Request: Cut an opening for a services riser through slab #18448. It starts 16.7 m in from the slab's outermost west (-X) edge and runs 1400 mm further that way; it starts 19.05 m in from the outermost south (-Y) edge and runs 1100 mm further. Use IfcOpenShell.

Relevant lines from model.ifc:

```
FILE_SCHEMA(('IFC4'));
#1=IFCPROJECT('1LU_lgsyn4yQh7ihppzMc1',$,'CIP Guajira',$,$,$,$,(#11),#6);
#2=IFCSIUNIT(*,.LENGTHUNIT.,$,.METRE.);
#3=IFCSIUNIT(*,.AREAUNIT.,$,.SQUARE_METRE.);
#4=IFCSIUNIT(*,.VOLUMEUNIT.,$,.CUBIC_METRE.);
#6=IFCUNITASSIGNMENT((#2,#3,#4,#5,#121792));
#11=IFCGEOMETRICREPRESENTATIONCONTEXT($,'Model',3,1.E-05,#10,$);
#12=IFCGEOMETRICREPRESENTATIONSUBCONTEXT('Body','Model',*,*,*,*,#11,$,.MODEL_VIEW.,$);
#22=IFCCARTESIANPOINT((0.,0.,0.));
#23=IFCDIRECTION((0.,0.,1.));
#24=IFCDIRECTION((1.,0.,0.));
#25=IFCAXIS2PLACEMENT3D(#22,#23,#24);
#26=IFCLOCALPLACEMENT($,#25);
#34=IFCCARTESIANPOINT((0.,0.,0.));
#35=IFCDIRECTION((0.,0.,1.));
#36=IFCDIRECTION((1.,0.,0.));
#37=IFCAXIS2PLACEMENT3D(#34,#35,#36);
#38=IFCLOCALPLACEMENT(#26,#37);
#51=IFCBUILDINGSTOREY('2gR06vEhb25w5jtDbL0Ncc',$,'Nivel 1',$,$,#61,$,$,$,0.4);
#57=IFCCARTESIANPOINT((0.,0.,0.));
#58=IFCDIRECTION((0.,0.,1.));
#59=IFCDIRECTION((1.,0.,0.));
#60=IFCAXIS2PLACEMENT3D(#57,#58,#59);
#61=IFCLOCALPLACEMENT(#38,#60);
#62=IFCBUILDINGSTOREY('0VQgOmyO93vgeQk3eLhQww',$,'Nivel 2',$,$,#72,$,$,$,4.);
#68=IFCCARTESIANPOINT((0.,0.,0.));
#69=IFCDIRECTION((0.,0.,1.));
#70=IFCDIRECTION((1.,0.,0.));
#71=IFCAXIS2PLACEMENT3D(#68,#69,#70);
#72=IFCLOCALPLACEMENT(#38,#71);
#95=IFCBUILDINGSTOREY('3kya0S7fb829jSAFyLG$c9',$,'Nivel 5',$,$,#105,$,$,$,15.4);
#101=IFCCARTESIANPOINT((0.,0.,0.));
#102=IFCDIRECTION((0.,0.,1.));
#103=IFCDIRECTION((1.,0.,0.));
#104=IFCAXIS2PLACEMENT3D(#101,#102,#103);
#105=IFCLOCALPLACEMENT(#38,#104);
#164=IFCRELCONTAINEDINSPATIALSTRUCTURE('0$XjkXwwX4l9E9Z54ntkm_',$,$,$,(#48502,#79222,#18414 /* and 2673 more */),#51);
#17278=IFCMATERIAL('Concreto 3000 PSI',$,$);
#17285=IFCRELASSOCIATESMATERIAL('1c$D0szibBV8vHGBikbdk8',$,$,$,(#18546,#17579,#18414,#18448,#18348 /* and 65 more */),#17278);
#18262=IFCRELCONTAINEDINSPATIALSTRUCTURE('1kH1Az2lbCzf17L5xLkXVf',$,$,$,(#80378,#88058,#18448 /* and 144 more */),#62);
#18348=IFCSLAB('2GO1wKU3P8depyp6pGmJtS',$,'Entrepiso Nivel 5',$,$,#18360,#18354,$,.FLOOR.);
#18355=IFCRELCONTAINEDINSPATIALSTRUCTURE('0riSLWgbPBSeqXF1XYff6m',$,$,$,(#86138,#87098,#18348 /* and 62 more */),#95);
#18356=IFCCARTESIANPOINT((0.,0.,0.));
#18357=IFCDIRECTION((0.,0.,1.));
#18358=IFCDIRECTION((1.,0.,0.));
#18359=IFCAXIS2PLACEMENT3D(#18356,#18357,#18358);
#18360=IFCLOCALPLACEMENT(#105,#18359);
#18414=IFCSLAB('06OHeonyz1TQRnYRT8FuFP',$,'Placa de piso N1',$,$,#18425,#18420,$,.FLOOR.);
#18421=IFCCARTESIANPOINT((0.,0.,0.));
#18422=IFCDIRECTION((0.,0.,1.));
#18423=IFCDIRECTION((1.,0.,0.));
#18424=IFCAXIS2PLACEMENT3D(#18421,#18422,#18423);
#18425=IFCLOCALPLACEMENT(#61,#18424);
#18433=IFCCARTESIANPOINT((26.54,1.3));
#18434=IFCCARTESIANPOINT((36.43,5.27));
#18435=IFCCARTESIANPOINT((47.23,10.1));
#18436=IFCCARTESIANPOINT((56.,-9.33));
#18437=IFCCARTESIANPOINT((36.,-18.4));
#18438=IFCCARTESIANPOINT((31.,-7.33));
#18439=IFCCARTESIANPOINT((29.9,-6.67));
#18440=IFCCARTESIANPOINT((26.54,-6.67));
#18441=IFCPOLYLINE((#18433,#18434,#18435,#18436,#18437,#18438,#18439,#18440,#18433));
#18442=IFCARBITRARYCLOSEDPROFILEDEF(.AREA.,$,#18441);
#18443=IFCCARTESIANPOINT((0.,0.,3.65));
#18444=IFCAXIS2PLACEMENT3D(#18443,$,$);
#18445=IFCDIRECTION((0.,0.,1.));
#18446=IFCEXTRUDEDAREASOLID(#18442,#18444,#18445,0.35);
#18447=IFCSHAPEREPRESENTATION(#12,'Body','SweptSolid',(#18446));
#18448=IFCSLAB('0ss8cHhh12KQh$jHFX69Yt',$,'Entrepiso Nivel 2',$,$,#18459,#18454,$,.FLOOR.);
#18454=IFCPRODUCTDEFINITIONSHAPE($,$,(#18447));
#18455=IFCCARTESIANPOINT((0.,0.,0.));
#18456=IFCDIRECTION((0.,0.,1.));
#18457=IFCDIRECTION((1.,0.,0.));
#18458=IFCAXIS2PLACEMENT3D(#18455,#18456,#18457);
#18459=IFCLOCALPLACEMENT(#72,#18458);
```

```python
import numpy as np
import ifcopenshell
import ifcopenshell.api.feature
import ifcopenshell.api.geometry
import ifcopenshell.api.root
import ifcopenshell.geom
import ifcopenshell.util.placement
import ifcopenshell.util.representation
import ifcopenshell.util.shape
import ifcopenshell.util.unit

model = ifcopenshell.open("model.ifc")
unit_scale = ifcopenshell.util.unit.calculate_unit_scale(model)
settings = ifcopenshell.geom.settings()


def volume(element):
    """Net volume in cubic metres, openings subtracted."""
    shape = ifcopenshell.geom.create_shape(settings, element)
    return ifcopenshell.util.shape.get_volume(shape.geometry)


slab = model.by_guid("0ss8cHhh12KQh$jHFX69Yt")
before = volume(slab)

# Extent in the slab's own axes, in metres. The edges named are its -X and -Y sides.
slab_shape = ifcopenshell.geom.create_shape(settings, slab)
vertices = ifcopenshell.util.shape.get_vertices(slab_shape.geometry)
x_min, y_min, bottom = vertices.min(axis=0)
top = vertices[:, 2].max()

opening = ifcopenshell.api.root.create_entity(model, ifc_class="IfcOpeningElement", name="Services riser opening", predefined_type="OPENING")
context = ifcopenshell.util.representation.get_context(model, "Model", "Body", "MODEL_VIEW")
width, depth = 1.4, 1.1
outline = [(0.0, 0.0), (width, 0.0), (width, depth), (0.0, depth), (0.0, 0.0)]
# Overshoot both faces by 50 mm so the cut is clean.
shape = ifcopenshell.api.geometry.add_slab_representation(
    model, context=context, depth=top - bottom + 0.1, polyline=outline
)
ifcopenshell.api.geometry.assign_representation(model, product=opening, representation=shape)

matrix = ifcopenshell.util.placement.get_local_placement(slab.ObjectPlacement)
matrix[:, 3] = matrix @ np.append(np.array([x_min + 16.7, y_min + 19.05, bottom - 0.05]) / unit_scale, 1.0)
ifcopenshell.api.geometry.edit_object_placement(model, product=opening, matrix=matrix, is_si=False)
ifcopenshell.api.feature.add_feature(model, feature=opening, element=slab)

after = volume(slab)

print(f"slab volume {before:.3f} -> {after:.3f} m3")

model.write("model_v2.ifc")
```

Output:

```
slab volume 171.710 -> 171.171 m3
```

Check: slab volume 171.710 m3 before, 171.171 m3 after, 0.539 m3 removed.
